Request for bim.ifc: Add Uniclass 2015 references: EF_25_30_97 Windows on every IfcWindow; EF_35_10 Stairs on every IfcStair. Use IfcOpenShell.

First a look at what the model holds.

```python
import ifcopenshell

model = ifcopenshell.open("bim.ifc")
print(model.schema)
print("classifications:", [c.Name for c in model.by_type("IfcClassification")])
for ifc_class in ("IfcDoor", "IfcRoof", "IfcStair", "IfcWall", "IfcWindow"):
    print(ifc_class, len(model.by_type(ifc_class)))
```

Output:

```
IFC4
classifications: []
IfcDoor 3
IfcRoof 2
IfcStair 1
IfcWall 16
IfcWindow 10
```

```python
import ifcopenshell
import ifcopenshell.api.classification

model = ifcopenshell.open("bim.ifc")

system = ifcopenshell.api.classification.add_classification(model, classification="Uniclass 2015")

codes = {
    "IfcWindow": ("EF_25_30_97", "Windows"),
    "IfcStair": ("EF_35_10", "Stairs"),
}
for ifc_class, (code, name) in codes.items():
    products = model.by_type(ifc_class)
    ifcopenshell.api.classification.add_reference(
        model, products=products, classification=system, identification=code, name=name
    )
    print(code, len(products))

model.write("bim_updated.ifc")
```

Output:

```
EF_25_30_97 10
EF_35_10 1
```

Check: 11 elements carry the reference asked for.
